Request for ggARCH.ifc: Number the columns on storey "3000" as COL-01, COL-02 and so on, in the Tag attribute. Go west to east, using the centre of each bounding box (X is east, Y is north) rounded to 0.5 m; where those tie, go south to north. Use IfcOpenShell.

First a look at what the model holds.

```python
import ifcopenshell
import ifcopenshell.util.element
import ifcopenshell.util.placement

model = ifcopenshell.open("ggARCH.ifc")
print(model.schema)
storey = next(s for s in model.by_type("IfcBuildingStorey") if s.Name == "3000")
columns = [e for e in ifcopenshell.util.element.get_decomposition(storey) if e.is_a("IfcColumn")]
for e in sorted(columns, key=lambda e: e.id()):
    origin = ifcopenshell.util.placement.get_local_placement(e.ObjectPlacement)[:3, 3]
    print(e.id(), e.Tag, e.Name, origin.round(2) + 0.0, sep=" | ")
```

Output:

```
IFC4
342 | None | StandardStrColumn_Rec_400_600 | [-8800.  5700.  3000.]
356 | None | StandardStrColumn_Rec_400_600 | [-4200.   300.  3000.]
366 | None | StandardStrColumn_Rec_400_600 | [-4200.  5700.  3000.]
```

```python
import ifcopenshell
import ifcopenshell.geom
import ifcopenshell.util.element
import ifcopenshell.util.shape

model = ifcopenshell.open("ggARCH.ifc")
settings = ifcopenshell.geom.settings()
settings.set("use-world-coords", True)


def centre(element):
    shape = ifcopenshell.geom.create_shape(settings, element)
    return ifcopenshell.util.shape.get_bbox_centroid(shape.geometry)


storey = next(s for s in model.by_type("IfcBuildingStorey") if s.Name == "3000")
columns = [e for e in ifcopenshell.util.element.get_decomposition(storey) if e.is_a("IfcColumn")]

# Insertion points can sit at a corner or the storey origin, so sort by the geometry (in metres).
centres = {e: centre(e) for e in columns}
columns.sort(key=lambda e: (round(centres[e][0] / 0.5), centres[e][1]))

for i, e in enumerate(columns, start=1):
    number = f"COL-{i:02d}"
    e.Tag = number
    print(e.id(), number)

model.write("ggARCH_rev.ifc")
```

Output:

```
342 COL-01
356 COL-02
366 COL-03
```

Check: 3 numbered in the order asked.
